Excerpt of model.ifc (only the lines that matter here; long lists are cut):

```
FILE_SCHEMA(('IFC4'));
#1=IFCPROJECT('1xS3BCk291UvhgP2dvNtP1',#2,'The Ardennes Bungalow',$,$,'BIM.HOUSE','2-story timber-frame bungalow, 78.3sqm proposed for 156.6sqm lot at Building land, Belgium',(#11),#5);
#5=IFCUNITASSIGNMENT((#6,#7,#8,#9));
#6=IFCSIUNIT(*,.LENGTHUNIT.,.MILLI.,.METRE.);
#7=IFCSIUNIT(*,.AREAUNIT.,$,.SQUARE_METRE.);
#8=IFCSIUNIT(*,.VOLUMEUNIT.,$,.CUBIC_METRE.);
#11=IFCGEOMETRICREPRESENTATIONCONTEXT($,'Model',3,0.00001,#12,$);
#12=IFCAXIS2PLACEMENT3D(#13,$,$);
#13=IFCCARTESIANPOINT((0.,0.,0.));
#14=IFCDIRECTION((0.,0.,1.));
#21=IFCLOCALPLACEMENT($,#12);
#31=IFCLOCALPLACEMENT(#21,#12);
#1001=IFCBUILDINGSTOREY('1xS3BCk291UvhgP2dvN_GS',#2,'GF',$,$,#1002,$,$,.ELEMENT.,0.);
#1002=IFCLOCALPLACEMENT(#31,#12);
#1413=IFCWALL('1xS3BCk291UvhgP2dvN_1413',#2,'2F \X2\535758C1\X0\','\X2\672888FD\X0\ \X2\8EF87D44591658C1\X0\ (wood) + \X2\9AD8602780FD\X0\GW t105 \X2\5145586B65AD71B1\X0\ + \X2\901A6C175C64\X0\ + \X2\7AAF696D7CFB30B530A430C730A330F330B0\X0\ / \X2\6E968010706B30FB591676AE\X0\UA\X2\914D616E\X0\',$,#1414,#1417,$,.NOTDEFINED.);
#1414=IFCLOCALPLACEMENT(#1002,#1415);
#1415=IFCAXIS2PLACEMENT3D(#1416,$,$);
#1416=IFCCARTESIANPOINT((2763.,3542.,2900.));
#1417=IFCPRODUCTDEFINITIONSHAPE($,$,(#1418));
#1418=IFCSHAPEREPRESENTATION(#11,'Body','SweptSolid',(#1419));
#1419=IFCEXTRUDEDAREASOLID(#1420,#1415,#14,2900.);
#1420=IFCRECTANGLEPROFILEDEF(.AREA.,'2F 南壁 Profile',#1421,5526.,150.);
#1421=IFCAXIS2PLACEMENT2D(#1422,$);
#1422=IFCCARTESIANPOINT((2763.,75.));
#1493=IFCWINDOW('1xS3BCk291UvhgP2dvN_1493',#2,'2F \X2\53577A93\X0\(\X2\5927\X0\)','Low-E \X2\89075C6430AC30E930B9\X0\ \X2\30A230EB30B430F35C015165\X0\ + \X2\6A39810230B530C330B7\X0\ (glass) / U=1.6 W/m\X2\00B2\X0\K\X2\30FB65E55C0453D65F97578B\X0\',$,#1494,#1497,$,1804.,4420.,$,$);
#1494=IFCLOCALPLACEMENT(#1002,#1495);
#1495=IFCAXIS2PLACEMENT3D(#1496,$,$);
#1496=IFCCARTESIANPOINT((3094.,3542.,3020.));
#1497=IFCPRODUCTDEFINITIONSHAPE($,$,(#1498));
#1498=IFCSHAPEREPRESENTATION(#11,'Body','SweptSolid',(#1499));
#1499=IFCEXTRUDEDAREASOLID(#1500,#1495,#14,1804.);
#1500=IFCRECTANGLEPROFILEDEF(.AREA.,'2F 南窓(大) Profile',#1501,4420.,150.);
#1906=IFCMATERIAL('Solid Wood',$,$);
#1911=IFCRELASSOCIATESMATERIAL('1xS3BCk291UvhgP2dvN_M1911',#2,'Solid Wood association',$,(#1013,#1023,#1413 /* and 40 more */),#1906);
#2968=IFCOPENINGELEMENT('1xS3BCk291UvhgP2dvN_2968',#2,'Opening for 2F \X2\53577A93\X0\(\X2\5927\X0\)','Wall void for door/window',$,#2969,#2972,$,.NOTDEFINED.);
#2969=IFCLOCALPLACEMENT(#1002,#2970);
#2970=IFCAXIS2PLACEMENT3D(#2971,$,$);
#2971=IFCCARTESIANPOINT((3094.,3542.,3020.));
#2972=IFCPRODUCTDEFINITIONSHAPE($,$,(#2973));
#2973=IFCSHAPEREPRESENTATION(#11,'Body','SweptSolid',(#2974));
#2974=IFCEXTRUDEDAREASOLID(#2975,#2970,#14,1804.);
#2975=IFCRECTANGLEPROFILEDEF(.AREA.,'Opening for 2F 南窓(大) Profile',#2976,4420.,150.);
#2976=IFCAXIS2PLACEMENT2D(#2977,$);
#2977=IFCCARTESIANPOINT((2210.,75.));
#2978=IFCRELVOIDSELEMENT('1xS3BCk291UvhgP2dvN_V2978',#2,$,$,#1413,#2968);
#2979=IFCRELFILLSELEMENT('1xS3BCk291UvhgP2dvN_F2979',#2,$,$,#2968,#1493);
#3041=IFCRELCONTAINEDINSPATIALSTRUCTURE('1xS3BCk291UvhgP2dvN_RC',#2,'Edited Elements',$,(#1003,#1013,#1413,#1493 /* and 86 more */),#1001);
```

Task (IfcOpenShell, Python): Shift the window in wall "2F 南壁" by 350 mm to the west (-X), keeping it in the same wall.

```python
import ifcopenshell
import ifcopenshell.api.geometry
import ifcopenshell.util.placement
import ifcopenshell.util.unit

model = ifcopenshell.open("model.ifc")
unit_scale = ifcopenshell.util.unit.calculate_unit_scale(model)

window = model.by_guid("1xS3BCk291UvhgP2dvN_1493")
opening = window.FillsVoids[0].RelatingOpeningElement
wall = opening.VoidsElements[0].RelatingBuildingElement

wall_matrix = ifcopenshell.util.placement.get_local_placement(wall.ObjectPlacement)
shift = wall_matrix[:3, 0] * -0.35 / unit_scale
before = ifcopenshell.util.placement.get_local_placement(window.ObjectPlacement)[:3, 3].copy()

# The window is not placed relative to its opening, so move both.
for product in (opening, window):
    matrix = ifcopenshell.util.placement.get_local_placement(product.ObjectPlacement)
    matrix[:3, 3] += shift
    ifcopenshell.api.geometry.edit_object_placement(model, product=product, matrix=matrix, is_si=False)

after = ifcopenshell.util.placement.get_local_placement(window.ObjectPlacement)[:3, 3]
print("window moved by", (after - before).round(3) + 0.0)

model.write("model_edited.ifc")
```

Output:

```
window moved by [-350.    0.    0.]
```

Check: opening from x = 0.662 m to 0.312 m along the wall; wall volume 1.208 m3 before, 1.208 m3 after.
